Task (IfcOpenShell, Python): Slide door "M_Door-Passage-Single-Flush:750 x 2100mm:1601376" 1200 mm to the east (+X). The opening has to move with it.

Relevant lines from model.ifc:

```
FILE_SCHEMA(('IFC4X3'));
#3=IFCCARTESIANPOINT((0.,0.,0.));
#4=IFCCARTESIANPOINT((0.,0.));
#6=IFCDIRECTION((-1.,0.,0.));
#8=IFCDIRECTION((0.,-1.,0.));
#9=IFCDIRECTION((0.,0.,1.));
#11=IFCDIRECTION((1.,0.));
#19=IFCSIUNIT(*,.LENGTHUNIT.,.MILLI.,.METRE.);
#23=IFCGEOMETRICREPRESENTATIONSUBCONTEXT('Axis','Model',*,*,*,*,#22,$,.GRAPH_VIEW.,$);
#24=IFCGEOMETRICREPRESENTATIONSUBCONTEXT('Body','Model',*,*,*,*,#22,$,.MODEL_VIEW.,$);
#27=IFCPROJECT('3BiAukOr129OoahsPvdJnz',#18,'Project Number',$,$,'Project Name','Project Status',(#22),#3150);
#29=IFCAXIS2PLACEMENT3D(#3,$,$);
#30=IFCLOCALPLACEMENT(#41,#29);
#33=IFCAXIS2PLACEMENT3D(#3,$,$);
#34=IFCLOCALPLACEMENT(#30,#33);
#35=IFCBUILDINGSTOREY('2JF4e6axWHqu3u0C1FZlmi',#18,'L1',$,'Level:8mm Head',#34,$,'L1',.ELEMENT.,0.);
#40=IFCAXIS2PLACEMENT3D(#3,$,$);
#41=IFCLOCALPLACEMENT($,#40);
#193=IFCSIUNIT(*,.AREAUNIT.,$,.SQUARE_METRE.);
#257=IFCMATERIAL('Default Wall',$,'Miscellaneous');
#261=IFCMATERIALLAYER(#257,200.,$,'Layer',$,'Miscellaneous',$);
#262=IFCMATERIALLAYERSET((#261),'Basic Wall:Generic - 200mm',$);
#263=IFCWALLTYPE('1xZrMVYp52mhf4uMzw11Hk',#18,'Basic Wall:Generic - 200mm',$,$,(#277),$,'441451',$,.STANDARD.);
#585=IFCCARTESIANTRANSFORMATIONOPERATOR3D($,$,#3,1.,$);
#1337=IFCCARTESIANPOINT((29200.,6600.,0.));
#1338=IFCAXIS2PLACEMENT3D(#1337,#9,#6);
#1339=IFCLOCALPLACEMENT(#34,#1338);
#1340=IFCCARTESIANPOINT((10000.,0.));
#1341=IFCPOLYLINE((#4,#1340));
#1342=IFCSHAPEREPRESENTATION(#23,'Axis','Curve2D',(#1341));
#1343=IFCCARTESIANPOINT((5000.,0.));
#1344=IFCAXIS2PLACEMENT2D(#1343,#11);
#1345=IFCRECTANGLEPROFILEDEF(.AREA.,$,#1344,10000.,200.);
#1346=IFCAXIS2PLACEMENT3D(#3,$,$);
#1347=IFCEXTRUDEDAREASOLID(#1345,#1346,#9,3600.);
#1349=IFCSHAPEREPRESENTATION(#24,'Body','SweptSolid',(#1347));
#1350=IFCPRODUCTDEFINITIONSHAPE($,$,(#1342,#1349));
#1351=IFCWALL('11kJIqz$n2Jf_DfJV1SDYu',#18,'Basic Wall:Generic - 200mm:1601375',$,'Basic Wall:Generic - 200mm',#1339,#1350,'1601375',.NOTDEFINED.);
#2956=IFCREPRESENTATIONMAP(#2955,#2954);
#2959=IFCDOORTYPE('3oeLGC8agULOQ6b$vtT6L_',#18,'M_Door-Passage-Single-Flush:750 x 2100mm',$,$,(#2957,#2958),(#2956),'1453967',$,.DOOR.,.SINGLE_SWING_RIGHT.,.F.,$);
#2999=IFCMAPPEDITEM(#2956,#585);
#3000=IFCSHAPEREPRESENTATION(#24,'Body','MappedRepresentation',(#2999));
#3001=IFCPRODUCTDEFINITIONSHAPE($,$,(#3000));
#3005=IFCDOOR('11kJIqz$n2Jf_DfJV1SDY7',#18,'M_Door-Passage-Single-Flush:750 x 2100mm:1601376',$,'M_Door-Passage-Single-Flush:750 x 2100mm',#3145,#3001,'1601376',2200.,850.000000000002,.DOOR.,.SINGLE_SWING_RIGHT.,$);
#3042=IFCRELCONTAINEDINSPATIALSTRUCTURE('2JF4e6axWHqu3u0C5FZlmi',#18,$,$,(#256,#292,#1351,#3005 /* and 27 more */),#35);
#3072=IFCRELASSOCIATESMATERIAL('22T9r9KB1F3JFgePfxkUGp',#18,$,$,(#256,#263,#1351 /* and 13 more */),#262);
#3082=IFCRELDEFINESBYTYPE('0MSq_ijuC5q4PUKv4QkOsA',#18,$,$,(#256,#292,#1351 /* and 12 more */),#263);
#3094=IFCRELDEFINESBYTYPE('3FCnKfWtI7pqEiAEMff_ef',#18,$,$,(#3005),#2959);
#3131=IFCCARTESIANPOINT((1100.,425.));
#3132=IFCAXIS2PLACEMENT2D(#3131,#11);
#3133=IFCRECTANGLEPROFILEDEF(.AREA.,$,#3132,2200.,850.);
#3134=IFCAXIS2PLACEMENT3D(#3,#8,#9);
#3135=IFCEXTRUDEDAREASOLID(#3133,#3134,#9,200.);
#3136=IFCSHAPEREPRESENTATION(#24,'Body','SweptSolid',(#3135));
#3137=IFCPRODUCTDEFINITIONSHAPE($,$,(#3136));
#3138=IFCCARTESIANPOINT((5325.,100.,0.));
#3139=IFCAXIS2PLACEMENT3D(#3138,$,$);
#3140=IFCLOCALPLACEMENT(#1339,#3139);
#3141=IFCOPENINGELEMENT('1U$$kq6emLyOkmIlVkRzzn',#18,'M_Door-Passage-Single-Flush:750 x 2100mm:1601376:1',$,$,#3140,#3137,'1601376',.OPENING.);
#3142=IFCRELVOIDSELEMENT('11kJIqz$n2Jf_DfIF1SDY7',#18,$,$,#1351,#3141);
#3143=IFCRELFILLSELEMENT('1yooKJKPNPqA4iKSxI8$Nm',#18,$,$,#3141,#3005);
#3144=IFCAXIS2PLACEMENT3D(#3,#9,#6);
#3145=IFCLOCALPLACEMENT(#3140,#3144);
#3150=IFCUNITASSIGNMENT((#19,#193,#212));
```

```python
import ifcopenshell
import ifcopenshell.api.geometry
import ifcopenshell.util.placement
import ifcopenshell.util.unit

model = ifcopenshell.open("model.ifc")
unit_scale = ifcopenshell.util.unit.calculate_unit_scale(model)

door = model.by_guid("11kJIqz$n2Jf_DfJV1SDY7")
opening = door.FillsVoids[0].RelatingOpeningElement
wall = opening.VoidsElements[0].RelatingBuildingElement

wall_matrix = ifcopenshell.util.placement.get_local_placement(wall.ObjectPlacement)
shift = wall_matrix[:3, 0] * -1.2 / unit_scale
before = ifcopenshell.util.placement.get_local_placement(door.ObjectPlacement)[:3, 3].copy()

# The door is placed relative to its opening, so it follows when the opening moves.
matrix = ifcopenshell.util.placement.get_local_placement(opening.ObjectPlacement)
matrix[:3, 3] += shift
ifcopenshell.api.geometry.edit_object_placement(
    model, product=opening, matrix=matrix, is_si=False, should_transform_children=True
)

after = ifcopenshell.util.placement.get_local_placement(door.ObjectPlacement)[:3, 3]
print("door moved by", (after - before).round(3) + 0.0)

model.write("model_updated.ifc")
```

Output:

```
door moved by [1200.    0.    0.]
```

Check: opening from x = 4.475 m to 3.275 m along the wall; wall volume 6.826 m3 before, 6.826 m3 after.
